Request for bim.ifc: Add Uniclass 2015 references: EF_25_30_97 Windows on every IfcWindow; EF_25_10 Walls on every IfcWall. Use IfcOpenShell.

First a look at what the model holds.

```python
import ifcopenshell

model = ifcopenshell.open("bim.ifc")
print(model.schema)
print("classifications:", [c.Name for c in model.by_type("IfcClassification")])
for ifc_class in ("IfcDoor", "IfcRoof", "IfcStair", "IfcWall", "IfcWindow"):
    print(ifc_class, len(model.by_type(ifc_class)))
```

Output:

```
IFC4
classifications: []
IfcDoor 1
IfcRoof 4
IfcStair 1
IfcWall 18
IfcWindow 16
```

```python
import ifcopenshell
import ifcopenshell.api.classification

model = ifcopenshell.open("bim.ifc")

system = ifcopenshell.api.classification.add_classification(model, classification="Uniclass 2015")

codes = {
    "IfcWindow": ("EF_25_30_97", "Windows"),
    "IfcWall": ("EF_25_10", "Walls"),
}
for ifc_class, (code, name) in codes.items():
    products = model.by_type(ifc_class)
    ifcopenshell.api.classification.add_reference(
        model, products=products, classification=system, identification=code, name=name
    )
    print(code, len(products))

model.write("bim_v2.ifc")
```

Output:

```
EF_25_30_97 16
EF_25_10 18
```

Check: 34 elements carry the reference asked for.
